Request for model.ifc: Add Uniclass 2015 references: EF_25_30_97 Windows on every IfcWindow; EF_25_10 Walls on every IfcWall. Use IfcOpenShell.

First a look at what the model holds.

```python
import ifcopenshell

model = ifcopenshell.open("model.ifc")
print(model.schema)
print("classifications:", [c.Name for c in model.by_type("IfcClassification")])
for ifc_class in ("IfcDoor", "IfcRoof", "IfcStair", "IfcWall", "IfcWindow"):
    print(ifc_class, len(model.by_type(ifc_class)))
```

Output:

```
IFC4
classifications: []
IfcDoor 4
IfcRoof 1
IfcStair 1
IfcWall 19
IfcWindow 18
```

```python
import ifcopenshell
import ifcopenshell.api.classification

model = ifcopenshell.open("model.ifc")

system = ifcopenshell.api.classification.add_classification(model, classification="Uniclass 2015")

codes = {
    "IfcWindow": ("EF_25_30_97", "Windows"),
    "IfcWall": ("EF_25_10", "Walls"),
}
for ifc_class, (code, name) in codes.items():
    products = model.by_type(ifc_class)
    ifcopenshell.api.classification.add_reference(
        model, products=products, classification=system, identification=code, name=name
    )
    print(code, len(products))

model.write("model_v2.ifc")
```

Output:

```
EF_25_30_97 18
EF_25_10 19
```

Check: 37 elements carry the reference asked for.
